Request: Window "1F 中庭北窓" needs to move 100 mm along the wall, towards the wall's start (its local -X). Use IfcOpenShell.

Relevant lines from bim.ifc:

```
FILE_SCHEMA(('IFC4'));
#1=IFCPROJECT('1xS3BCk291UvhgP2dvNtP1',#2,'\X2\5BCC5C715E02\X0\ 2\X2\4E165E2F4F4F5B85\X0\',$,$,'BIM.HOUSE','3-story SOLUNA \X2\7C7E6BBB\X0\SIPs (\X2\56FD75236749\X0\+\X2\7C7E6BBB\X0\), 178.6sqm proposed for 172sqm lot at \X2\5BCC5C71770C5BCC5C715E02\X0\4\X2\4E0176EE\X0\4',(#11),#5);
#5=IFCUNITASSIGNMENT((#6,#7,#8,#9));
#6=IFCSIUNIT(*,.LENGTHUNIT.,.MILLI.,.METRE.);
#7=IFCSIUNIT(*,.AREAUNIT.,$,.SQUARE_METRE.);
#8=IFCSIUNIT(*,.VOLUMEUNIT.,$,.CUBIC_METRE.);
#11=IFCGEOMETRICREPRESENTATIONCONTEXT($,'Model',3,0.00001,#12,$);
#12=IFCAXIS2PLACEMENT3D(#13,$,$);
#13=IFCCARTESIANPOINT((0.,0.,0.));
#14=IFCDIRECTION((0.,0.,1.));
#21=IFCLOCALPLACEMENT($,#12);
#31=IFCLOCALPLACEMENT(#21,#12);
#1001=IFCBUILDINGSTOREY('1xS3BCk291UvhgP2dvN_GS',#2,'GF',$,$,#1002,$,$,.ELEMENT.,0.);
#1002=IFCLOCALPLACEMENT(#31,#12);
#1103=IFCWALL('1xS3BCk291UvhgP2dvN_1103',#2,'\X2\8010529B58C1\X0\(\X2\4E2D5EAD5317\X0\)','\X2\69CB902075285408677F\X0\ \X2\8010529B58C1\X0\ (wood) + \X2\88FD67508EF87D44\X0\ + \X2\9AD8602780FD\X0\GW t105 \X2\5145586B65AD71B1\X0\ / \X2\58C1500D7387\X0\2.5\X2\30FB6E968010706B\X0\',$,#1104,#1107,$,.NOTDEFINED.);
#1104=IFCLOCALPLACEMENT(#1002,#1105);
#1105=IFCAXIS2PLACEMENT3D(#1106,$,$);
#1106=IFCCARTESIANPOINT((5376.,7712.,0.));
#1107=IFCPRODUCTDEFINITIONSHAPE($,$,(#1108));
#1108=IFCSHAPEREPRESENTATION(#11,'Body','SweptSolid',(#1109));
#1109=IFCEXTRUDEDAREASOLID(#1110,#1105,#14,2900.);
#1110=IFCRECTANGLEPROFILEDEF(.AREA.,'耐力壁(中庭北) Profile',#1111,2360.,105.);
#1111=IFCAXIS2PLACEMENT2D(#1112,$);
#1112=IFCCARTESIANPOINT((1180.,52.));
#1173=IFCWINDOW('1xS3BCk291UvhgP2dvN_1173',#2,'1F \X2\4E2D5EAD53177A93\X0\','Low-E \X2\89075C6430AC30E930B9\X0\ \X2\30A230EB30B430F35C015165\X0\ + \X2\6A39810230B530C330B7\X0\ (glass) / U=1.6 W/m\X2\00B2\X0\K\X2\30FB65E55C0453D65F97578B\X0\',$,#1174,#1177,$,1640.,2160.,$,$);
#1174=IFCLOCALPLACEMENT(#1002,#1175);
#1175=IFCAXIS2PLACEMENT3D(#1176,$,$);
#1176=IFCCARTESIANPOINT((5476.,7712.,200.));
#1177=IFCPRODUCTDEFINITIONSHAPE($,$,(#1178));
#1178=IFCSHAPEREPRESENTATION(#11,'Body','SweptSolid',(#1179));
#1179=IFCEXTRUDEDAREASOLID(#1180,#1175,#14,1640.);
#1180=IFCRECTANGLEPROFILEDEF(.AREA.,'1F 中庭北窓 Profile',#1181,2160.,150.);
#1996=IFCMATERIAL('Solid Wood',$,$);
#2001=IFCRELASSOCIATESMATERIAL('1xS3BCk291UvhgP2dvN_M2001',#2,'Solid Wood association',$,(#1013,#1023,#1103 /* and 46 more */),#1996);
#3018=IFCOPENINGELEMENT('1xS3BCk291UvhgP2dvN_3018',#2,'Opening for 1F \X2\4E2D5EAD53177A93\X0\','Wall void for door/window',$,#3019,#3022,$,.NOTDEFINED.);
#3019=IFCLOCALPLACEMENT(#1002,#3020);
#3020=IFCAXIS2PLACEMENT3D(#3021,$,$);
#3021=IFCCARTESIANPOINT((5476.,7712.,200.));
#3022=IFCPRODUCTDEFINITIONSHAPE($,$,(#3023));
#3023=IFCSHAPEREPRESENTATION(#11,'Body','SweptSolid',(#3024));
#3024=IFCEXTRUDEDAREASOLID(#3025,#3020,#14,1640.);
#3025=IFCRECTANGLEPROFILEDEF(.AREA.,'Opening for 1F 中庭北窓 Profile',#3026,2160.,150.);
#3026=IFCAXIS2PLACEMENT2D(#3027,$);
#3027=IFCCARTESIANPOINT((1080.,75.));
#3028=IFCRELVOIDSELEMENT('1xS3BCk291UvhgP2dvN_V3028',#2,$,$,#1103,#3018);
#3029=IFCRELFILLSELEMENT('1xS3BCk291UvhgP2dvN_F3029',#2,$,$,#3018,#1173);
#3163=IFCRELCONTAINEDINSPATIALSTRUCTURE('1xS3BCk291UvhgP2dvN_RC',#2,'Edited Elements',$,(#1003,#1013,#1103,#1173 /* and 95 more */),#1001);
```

```python
import ifcopenshell
import ifcopenshell.api.geometry
import ifcopenshell.util.placement
import ifcopenshell.util.unit

model = ifcopenshell.open("bim.ifc")
unit_scale = ifcopenshell.util.unit.calculate_unit_scale(model)

window = model.by_guid("1xS3BCk291UvhgP2dvN_1173")
opening = window.FillsVoids[0].RelatingOpeningElement
wall = opening.VoidsElements[0].RelatingBuildingElement

wall_matrix = ifcopenshell.util.placement.get_local_placement(wall.ObjectPlacement)
shift = wall_matrix[:3, 0] * -0.1 / unit_scale
before = ifcopenshell.util.placement.get_local_placement(window.ObjectPlacement)[:3, 3].copy()

# The window is not placed relative to its opening, so move both.
for product in (opening, window):
    matrix = ifcopenshell.util.placement.get_local_placement(product.ObjectPlacement)
    matrix[:3, 3] += shift
    ifcopenshell.api.geometry.edit_object_placement(model, product=product, matrix=matrix, is_si=False)

after = ifcopenshell.util.placement.get_local_placement(window.ObjectPlacement)[:3, 3]
print("window moved by", (after - before).round(3) + 0.0)

model.write("bim_rev.ifc")
```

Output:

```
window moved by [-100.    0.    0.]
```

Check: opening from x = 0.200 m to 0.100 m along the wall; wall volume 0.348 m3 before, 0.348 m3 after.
